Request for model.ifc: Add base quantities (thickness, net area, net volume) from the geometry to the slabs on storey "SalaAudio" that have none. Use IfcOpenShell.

First a look at what the model holds.

```python
import ifcopenshell
import ifcopenshell.util.element
import ifcopenshell.util.unit

model = ifcopenshell.open("model.ifc")
print(model.schema)
for unit_type in ("LENGTHUNIT", "AREAUNIT", "VOLUMEUNIT"):
    print(unit_type, ifcopenshell.util.unit.calculate_unit_scale(model, unit_type))
storey = next(s for s in model.by_type("IfcBuildingStorey") if s.Name == "SalaAudio")
slabs = [e for e in ifcopenshell.util.element.get_decomposition(storey) if e.is_a("IfcSlab")]
for e in sorted(slabs, key=lambda e: e.id()):
    print(e.id(), e.is_a(), e.Name, list(ifcopenshell.util.element.get_psets(e, qtos_only=True)), sep=" | ")
```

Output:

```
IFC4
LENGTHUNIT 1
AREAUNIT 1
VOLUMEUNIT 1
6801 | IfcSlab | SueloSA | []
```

```python
import ifcopenshell
import ifcopenshell.api.pset
import ifcopenshell.geom
import ifcopenshell.util.element
import ifcopenshell.util.shape
import ifcopenshell.util.unit

model = ifcopenshell.open("model.ifc")
unit_scale = ifcopenshell.util.unit.calculate_unit_scale(model)
area_scale = ifcopenshell.util.unit.calculate_unit_scale(model, "AREAUNIT")
volume_scale = ifcopenshell.util.unit.calculate_unit_scale(model, "VOLUMEUNIT")
settings = ifcopenshell.geom.settings()

storey = next(s for s in model.by_type("IfcBuildingStorey") if s.Name == "SalaAudio")
slabs = [e for e in ifcopenshell.util.element.get_decomposition(storey) if e.is_a("IfcSlab")]

for e in sorted(slabs, key=lambda e: e.id()):
    if ifcopenshell.util.element.get_psets(e, qtos_only=True, should_inherit=False):
        continue
    # Geometry comes back in metres, in the element's own axes.
    shape = ifcopenshell.geom.create_shape(settings, e)
    values = {
        "Width": ifcopenshell.util.shape.get_z(shape.geometry) / unit_scale,
        "NetArea": ifcopenshell.util.shape.get_footprint_area(shape.geometry) / area_scale,
        "NetVolume": ifcopenshell.util.shape.get_volume(shape.geometry) / volume_scale,
    }
    qto = ifcopenshell.api.pset.add_qto(model, product=e, name="Qto_SlabBaseQuantities")
    ifcopenshell.api.pset.edit_qto(model, qto=qto, properties=values)
    print(e.id(), {k: round(v, 3) for k, v in values.items()})

model.write("model_edited.ifc")
```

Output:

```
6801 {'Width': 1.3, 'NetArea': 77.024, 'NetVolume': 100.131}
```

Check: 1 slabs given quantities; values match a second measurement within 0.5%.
